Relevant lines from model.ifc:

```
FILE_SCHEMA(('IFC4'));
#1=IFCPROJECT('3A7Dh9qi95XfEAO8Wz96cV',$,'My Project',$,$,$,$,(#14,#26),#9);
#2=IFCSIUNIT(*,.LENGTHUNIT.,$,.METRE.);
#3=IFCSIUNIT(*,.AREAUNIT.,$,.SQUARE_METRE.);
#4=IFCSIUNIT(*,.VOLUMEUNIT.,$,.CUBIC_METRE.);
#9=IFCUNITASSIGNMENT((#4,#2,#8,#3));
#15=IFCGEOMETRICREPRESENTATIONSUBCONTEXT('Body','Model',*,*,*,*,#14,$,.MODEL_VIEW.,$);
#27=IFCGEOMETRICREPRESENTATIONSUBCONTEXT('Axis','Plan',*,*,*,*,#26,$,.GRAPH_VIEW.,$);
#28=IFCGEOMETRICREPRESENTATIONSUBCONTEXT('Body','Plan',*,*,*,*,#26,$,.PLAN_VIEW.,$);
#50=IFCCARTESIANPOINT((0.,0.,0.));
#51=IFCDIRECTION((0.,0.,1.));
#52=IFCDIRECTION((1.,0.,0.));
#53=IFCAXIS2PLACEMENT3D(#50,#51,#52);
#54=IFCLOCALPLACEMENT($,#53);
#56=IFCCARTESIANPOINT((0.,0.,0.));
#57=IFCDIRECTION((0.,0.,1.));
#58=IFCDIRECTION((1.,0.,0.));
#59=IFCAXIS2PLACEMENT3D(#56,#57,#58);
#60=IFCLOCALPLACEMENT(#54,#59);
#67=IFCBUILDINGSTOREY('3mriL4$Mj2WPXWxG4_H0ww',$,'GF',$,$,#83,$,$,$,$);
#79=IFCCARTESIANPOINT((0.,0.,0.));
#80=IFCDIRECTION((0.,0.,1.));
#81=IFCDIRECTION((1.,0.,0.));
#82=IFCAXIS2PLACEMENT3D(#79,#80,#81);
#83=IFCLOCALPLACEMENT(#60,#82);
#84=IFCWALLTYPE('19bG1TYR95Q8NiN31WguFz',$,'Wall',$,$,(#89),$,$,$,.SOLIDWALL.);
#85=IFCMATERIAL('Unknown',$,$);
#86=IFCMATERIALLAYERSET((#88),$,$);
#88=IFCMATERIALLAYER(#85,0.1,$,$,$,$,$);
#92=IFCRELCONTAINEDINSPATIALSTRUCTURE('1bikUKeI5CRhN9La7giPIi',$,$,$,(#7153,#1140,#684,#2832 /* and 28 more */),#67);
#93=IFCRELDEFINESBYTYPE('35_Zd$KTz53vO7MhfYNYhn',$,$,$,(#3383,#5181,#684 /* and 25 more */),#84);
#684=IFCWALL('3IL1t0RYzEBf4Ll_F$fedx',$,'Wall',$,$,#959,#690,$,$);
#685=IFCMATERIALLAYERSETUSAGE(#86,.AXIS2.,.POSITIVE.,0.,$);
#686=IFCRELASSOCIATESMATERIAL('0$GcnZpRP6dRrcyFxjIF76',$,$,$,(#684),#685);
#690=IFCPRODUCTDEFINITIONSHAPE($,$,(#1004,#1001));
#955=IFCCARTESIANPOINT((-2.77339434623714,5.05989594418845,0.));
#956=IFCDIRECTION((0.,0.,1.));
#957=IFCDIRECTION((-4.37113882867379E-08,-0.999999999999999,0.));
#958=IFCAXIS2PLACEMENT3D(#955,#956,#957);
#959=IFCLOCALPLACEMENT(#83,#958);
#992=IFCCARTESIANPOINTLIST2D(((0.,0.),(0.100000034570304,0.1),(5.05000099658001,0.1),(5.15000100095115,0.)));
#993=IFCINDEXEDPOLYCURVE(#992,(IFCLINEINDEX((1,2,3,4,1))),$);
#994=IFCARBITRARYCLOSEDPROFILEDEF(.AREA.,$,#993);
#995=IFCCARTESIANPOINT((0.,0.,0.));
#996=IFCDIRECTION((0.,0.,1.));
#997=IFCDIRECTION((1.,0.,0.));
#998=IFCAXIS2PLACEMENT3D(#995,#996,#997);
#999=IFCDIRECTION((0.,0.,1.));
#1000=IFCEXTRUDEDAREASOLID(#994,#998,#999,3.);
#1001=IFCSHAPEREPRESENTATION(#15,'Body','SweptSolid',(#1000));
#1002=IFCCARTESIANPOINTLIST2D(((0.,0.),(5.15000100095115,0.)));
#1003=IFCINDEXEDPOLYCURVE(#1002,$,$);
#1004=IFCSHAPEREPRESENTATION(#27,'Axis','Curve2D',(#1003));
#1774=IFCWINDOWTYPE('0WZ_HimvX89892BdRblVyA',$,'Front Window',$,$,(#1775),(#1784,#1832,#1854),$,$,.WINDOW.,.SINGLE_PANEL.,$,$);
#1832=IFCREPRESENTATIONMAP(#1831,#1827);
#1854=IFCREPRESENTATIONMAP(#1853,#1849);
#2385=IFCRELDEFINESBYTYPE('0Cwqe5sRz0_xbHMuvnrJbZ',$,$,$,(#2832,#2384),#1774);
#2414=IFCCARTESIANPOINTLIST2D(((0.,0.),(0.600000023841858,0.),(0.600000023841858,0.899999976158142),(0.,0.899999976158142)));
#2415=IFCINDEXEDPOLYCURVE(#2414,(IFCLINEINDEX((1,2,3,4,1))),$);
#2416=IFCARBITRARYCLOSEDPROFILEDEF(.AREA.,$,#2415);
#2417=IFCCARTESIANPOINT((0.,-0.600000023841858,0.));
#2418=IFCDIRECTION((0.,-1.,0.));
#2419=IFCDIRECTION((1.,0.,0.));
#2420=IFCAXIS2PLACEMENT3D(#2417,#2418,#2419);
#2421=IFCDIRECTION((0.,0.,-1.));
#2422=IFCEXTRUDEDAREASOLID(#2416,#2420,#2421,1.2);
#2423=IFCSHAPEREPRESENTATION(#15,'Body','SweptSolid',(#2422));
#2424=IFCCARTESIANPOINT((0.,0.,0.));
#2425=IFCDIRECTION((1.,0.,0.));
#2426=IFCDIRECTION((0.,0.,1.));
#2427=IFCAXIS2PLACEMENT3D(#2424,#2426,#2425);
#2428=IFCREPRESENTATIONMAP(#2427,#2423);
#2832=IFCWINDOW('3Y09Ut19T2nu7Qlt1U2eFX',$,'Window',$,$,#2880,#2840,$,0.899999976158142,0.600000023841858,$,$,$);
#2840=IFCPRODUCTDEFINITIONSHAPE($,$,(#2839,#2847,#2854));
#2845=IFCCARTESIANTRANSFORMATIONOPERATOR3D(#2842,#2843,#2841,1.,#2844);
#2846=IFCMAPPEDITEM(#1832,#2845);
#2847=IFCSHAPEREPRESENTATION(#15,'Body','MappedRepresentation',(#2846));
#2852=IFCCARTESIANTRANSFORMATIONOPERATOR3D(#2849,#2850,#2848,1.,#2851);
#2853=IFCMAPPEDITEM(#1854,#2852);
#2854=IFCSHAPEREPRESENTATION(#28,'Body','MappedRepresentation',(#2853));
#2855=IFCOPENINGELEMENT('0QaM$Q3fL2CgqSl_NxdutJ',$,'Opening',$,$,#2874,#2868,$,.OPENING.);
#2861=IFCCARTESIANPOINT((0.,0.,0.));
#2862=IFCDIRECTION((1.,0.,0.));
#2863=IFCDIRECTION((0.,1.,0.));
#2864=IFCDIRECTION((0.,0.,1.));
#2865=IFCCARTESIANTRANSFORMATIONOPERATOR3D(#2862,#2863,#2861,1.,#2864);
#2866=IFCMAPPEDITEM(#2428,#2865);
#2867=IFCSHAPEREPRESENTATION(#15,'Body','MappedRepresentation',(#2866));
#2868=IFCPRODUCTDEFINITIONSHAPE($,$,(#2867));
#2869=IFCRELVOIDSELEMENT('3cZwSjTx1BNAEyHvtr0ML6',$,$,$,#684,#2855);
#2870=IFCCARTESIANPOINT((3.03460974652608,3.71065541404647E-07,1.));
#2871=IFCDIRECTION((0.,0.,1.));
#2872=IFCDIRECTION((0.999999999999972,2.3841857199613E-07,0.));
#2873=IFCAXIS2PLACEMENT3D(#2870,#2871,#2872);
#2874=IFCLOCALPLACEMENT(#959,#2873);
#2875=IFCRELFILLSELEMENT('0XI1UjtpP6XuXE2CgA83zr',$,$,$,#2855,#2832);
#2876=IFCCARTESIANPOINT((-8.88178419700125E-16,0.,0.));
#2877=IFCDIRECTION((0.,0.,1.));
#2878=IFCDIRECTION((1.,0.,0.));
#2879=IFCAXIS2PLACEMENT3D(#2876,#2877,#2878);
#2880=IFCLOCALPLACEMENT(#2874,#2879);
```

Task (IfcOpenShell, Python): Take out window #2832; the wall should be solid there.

```python
import ifcopenshell
import ifcopenshell.api.feature
import ifcopenshell.api.root
import ifcopenshell.geom
import ifcopenshell.util.shape

model = ifcopenshell.open("model.ifc")
settings = ifcopenshell.geom.settings()


def volume(element):
    """Net volume in cubic metres, openings subtracted."""
    shape = ifcopenshell.geom.create_shape(settings, element)
    return ifcopenshell.util.shape.get_volume(shape.geometry)


window = model.by_guid("3Y09Ut19T2nu7Qlt1U2eFX")
opening = window.FillsVoids[0].RelatingOpeningElement
wall = opening.VoidsElements[0].RelatingBuildingElement
before = volume(wall)

ifcopenshell.api.root.remove_product(model, product=window)
ifcopenshell.api.feature.remove_feature(model, feature=opening)

after = volume(wall)

print(f"wall volume {before:.3f} -> {after:.3f} m3")

model.write("model_edited.ifc")
```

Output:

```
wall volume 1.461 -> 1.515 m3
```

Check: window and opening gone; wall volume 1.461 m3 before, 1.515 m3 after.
